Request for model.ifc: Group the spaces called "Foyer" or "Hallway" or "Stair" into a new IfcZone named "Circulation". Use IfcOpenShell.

First a look at what the model holds.

```python
import ifcopenshell

model = ifcopenshell.open("model.ifc")
print(model.schema)
seen = {}
for space in model.by_type("IfcSpace"):
    seen[space.LongName] = seen.get(space.LongName, 0) + 1
for name, count in sorted(seen.items(), key=str):
    print(count, "x", name)
print("zones:", [z.Name for z in model.by_type("IfcZone")][:20])
```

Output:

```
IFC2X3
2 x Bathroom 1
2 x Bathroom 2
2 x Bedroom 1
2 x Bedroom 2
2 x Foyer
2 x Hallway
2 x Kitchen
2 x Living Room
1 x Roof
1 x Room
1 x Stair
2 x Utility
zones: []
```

```python
import ifcopenshell
import ifcopenshell.api.group
import ifcopenshell.api.root

model = ifcopenshell.open("model.ifc")

names = {"Foyer", "Hallway", "Stair"}
spaces = [s for s in model.by_type("IfcSpace") if s.LongName in names]

zone = ifcopenshell.api.root.create_entity(model, ifc_class="IfcZone", name="Circulation")
ifcopenshell.api.group.assign_group(model, products=spaces, group=zone)
print(len(spaces), "spaces in", zone.Name)

model.write("model_updated.ifc")
```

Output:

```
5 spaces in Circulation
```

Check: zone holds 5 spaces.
